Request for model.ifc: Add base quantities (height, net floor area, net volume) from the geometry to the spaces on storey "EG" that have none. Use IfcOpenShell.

First a look at what the model holds.

```python
import ifcopenshell
import ifcopenshell.util.element
import ifcopenshell.util.unit

model = ifcopenshell.open("model.ifc")
print(model.schema)
for unit_type in ("LENGTHUNIT", "AREAUNIT", "VOLUMEUNIT"):
    print(unit_type, ifcopenshell.util.unit.calculate_unit_scale(model, unit_type))
storey = next(s for s in model.by_type("IfcBuildingStorey") if s.Name == "EG")
spaces = [e for e in ifcopenshell.util.element.get_decomposition(storey) if e.is_a("IfcSpace")]
for e in sorted(spaces, key=lambda e: e.id()):
    print(e.id(), e.is_a(), e.Name, list(ifcopenshell.util.element.get_psets(e, qtos_only=True)), sep=" | ")
```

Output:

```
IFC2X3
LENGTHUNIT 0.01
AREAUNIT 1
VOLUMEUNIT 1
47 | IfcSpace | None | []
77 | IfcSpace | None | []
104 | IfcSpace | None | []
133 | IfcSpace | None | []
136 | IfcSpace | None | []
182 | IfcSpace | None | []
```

```python
import ifcopenshell
import ifcopenshell.api.pset
import ifcopenshell.geom
import ifcopenshell.util.element
import ifcopenshell.util.shape
import ifcopenshell.util.unit

model = ifcopenshell.open("model.ifc")
unit_scale = ifcopenshell.util.unit.calculate_unit_scale(model)
area_scale = ifcopenshell.util.unit.calculate_unit_scale(model, "AREAUNIT")
volume_scale = ifcopenshell.util.unit.calculate_unit_scale(model, "VOLUMEUNIT")
settings = ifcopenshell.geom.settings()

storey = next(s for s in model.by_type("IfcBuildingStorey") if s.Name == "EG")
spaces = [e for e in ifcopenshell.util.element.get_decomposition(storey) if e.is_a("IfcSpace")]

for e in sorted(spaces, key=lambda e: e.id()):
    if ifcopenshell.util.element.get_psets(e, qtos_only=True, should_inherit=False):
        continue
    # Geometry comes back in metres, in the element's own axes.
    shape = ifcopenshell.geom.create_shape(settings, e)
    values = {
        "Height": ifcopenshell.util.shape.get_z(shape.geometry) / unit_scale,
        "NetFloorArea": ifcopenshell.util.shape.get_footprint_area(shape.geometry) / area_scale,
        "NetVolume": ifcopenshell.util.shape.get_volume(shape.geometry) / volume_scale,
    }
    qto = ifcopenshell.api.pset.add_qto(model, product=e, name="BaseQuantities")
    ifcopenshell.api.pset.edit_qto(model, qto=qto, properties=values)
    print(e.id(), {k: round(v, 3) for k, v in values.items()})

model.write("model_rev.ifc")
```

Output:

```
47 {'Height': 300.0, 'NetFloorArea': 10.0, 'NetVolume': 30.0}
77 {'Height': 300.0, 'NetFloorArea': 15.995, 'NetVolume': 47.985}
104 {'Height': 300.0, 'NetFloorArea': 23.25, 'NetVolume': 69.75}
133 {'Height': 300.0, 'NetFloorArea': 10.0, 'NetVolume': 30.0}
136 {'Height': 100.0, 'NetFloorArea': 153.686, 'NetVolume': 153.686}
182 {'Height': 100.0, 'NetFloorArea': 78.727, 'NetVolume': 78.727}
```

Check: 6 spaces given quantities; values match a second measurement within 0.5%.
